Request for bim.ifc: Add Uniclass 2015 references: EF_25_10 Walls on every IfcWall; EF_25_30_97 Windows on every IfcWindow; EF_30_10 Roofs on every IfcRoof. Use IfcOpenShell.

First a look at what the model holds.

```python
import ifcopenshell

model = ifcopenshell.open("bim.ifc")
print(model.schema)
print("classifications:", [c.Name for c in model.by_type("IfcClassification")])
for ifc_class in ("IfcDoor", "IfcRoof", "IfcStair", "IfcWall", "IfcWindow"):
    print(ifc_class, len(model.by_type(ifc_class)))
```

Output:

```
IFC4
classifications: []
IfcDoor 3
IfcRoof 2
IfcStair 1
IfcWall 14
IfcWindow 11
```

```python
import ifcopenshell
import ifcopenshell.api.classification

model = ifcopenshell.open("bim.ifc")

system = ifcopenshell.api.classification.add_classification(model, classification="Uniclass 2015")

codes = {
    "IfcWall": ("EF_25_10", "Walls"),
    "IfcWindow": ("EF_25_30_97", "Windows"),
    "IfcRoof": ("EF_30_10", "Roofs"),
}
for ifc_class, (code, name) in codes.items():
    products = model.by_type(ifc_class)
    ifcopenshell.api.classification.add_reference(
        model, products=products, classification=system, identification=code, name=name
    )
    print(code, len(products))

model.write("bim_edited.ifc")
```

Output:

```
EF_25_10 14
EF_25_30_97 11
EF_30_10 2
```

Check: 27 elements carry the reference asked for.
